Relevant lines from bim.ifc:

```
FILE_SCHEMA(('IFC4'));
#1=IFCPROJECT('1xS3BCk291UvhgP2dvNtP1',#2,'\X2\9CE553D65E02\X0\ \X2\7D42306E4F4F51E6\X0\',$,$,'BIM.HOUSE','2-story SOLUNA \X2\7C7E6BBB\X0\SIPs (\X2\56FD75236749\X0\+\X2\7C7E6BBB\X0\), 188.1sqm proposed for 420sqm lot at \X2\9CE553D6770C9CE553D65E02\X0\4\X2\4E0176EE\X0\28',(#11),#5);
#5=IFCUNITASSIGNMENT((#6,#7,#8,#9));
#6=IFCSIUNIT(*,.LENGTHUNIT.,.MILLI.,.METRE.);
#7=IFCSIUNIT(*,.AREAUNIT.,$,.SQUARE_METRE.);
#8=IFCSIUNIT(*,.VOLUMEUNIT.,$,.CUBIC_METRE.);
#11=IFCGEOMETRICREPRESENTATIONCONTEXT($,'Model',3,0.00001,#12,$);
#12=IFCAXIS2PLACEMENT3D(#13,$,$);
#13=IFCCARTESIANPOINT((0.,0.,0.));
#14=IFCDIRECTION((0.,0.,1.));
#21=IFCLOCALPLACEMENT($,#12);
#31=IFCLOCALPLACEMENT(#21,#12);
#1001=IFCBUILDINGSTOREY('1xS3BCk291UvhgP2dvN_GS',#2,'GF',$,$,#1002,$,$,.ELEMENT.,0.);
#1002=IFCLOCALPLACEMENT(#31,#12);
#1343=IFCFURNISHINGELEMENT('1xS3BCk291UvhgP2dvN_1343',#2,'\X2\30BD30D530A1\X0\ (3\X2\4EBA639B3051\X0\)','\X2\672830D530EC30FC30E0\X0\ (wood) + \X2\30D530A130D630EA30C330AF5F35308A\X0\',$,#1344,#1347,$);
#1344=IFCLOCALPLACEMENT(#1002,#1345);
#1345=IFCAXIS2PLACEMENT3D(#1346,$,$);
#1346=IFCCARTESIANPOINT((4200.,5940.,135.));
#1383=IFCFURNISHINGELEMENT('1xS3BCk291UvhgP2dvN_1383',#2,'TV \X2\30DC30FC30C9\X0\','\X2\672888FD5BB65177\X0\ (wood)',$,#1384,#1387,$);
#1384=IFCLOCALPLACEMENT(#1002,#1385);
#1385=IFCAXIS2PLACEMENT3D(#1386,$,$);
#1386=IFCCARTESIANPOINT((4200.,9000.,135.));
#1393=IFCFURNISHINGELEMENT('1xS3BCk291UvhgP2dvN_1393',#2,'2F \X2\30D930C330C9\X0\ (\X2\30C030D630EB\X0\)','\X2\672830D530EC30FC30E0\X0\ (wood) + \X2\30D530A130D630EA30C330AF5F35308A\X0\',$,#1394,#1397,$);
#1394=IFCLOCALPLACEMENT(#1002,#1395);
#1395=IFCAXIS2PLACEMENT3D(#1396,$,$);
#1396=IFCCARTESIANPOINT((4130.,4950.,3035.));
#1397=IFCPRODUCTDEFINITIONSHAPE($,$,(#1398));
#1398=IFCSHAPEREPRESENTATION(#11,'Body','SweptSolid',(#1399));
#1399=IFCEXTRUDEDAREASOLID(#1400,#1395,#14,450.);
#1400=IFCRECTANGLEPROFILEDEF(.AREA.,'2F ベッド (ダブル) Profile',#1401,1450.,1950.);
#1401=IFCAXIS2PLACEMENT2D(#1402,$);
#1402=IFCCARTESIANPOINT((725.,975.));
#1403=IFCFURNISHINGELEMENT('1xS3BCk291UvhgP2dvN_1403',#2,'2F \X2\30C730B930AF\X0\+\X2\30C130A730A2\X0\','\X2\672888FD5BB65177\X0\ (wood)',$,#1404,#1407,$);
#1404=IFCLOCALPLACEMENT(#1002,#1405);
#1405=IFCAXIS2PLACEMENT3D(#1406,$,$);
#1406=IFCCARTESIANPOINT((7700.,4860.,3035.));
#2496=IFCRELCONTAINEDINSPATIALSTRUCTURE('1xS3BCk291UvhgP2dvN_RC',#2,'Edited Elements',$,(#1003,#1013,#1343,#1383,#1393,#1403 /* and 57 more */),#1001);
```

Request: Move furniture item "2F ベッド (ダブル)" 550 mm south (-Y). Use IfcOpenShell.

```python
import ifcopenshell
import ifcopenshell.api.geometry
import ifcopenshell.util.placement
import ifcopenshell.util.unit

model = ifcopenshell.open("bim.ifc")
unit_scale = ifcopenshell.util.unit.calculate_unit_scale(model)

item = model.by_guid("1xS3BCk291UvhgP2dvN_1393")
matrix = ifcopenshell.util.placement.get_local_placement(item.ObjectPlacement)
matrix[1, 3] -= 0.55 / unit_scale
ifcopenshell.api.geometry.edit_object_placement(model, product=item, matrix=matrix, is_si=False)

print(ifcopenshell.util.placement.get_local_placement(item.ObjectPlacement).round(3) + 0.0)

model.write("bim_v2.ifc")
```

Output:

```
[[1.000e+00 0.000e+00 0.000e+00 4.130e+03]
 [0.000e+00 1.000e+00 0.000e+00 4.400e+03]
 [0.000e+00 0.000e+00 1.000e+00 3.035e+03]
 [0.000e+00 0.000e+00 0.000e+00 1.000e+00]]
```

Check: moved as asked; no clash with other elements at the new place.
